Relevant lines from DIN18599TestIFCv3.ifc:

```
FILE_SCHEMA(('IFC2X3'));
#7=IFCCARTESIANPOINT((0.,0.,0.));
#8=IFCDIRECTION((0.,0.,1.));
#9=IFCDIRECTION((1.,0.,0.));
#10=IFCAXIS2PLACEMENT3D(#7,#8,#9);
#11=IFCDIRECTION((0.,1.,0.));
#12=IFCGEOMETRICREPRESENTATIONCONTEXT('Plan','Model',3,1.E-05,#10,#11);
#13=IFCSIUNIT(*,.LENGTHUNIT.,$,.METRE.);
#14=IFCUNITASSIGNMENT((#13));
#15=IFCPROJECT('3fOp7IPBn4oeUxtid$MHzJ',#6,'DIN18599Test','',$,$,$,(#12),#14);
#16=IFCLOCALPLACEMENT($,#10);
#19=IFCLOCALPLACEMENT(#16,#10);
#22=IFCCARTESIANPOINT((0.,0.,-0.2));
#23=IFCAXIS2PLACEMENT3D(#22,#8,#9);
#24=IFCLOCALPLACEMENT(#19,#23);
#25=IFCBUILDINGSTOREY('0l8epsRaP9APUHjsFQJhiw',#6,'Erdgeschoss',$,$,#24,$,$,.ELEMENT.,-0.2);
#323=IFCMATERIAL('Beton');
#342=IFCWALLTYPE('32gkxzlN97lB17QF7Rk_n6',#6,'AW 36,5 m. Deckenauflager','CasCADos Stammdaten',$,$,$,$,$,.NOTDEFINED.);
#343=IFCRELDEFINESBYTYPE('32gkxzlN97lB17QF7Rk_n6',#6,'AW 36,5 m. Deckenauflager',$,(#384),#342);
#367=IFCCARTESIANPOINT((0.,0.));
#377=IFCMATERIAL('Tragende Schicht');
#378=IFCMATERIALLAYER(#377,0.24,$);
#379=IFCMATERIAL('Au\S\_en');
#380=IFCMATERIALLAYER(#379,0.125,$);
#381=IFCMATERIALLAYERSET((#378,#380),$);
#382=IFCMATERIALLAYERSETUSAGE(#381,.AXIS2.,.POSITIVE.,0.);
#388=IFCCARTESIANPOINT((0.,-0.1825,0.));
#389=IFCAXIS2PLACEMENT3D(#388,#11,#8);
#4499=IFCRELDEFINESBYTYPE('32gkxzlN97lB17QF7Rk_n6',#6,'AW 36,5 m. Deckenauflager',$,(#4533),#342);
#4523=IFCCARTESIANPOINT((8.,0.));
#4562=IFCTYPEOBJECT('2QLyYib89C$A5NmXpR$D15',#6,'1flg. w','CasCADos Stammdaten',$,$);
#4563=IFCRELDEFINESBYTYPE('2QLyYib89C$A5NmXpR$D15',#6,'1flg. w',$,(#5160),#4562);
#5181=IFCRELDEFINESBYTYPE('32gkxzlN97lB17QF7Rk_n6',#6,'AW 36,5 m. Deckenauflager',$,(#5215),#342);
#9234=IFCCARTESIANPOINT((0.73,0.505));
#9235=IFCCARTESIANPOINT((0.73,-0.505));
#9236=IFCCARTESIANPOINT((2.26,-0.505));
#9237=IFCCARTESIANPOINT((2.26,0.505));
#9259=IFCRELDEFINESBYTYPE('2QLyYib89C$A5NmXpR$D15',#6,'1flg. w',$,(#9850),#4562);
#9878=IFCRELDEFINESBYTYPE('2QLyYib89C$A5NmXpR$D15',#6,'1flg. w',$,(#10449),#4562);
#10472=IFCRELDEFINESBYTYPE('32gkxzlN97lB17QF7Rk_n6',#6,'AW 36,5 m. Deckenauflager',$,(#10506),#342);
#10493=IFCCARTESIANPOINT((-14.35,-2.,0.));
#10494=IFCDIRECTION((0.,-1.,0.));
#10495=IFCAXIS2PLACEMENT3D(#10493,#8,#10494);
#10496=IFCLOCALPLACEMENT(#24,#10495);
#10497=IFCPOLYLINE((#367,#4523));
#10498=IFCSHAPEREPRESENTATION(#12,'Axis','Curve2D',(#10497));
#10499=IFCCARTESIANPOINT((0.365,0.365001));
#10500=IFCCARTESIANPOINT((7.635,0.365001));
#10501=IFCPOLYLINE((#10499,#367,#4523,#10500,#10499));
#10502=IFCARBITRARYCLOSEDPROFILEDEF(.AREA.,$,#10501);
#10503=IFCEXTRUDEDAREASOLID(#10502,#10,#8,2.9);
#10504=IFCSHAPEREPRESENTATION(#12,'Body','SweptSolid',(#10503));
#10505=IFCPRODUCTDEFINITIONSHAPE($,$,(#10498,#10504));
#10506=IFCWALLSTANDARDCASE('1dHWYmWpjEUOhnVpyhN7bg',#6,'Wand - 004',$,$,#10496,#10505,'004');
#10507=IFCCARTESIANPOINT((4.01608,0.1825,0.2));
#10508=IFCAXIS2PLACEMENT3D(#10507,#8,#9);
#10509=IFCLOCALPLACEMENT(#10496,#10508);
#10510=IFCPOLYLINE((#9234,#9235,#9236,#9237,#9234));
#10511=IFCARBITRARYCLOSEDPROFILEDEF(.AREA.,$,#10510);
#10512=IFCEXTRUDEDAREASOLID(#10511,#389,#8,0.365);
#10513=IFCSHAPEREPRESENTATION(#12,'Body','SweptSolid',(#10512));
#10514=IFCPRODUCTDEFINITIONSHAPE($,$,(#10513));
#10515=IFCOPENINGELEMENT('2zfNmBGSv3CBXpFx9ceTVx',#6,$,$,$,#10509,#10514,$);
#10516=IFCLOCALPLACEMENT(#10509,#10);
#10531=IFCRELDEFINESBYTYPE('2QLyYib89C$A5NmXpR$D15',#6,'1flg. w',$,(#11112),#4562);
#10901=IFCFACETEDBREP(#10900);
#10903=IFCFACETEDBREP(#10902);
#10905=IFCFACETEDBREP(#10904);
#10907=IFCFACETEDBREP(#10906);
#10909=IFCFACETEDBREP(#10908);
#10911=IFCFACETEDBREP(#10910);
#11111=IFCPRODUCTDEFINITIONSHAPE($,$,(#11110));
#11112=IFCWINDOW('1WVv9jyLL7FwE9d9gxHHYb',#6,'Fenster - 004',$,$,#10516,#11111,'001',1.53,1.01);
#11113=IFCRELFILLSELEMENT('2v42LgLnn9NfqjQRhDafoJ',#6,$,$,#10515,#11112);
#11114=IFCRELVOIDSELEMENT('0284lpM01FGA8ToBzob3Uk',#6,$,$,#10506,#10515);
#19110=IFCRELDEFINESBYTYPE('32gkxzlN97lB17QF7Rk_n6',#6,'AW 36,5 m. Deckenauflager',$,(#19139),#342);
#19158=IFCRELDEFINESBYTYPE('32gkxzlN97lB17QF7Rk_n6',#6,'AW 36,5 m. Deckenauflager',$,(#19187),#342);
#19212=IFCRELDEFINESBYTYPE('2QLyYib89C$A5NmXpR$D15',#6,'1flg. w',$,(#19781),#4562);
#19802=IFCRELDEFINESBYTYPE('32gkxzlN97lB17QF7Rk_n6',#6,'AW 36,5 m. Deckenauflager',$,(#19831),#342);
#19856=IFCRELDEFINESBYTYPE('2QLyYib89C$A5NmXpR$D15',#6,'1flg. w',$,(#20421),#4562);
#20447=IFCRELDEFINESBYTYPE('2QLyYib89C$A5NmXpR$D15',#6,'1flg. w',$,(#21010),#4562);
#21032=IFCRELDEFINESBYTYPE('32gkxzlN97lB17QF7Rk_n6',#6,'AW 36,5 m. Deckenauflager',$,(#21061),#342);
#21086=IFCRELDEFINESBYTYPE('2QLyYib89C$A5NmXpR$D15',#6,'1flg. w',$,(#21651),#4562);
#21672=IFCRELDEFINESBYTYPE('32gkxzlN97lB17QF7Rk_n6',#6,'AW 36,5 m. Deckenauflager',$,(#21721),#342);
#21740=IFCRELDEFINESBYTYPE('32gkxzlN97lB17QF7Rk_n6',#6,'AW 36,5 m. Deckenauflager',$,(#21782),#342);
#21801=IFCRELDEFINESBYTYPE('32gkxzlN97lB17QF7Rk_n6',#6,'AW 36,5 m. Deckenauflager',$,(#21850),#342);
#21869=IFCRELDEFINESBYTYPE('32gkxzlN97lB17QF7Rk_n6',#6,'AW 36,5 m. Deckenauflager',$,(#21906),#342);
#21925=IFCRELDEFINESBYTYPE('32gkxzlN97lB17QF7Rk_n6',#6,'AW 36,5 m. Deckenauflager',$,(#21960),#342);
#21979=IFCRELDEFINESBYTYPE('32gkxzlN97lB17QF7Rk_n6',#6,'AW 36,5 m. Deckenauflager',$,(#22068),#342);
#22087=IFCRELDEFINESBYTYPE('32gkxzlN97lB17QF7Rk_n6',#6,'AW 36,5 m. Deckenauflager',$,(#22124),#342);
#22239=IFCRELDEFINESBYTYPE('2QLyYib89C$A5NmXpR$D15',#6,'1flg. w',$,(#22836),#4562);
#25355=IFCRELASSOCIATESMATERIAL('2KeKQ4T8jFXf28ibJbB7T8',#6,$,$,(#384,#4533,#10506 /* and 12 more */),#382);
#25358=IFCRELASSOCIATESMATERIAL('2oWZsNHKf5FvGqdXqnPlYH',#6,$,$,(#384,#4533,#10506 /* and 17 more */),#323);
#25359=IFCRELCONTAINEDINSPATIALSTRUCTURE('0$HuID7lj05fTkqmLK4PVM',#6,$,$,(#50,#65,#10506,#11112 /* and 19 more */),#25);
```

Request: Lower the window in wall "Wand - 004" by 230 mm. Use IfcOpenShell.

```python
import numpy as np
import ifcopenshell
import ifcopenshell.api.geometry
import ifcopenshell.util.placement
import ifcopenshell.util.unit

model = ifcopenshell.open("DIN18599TestIFCv3.ifc")
unit_scale = ifcopenshell.util.unit.calculate_unit_scale(model)

window = model.by_guid("1WVv9jyLL7FwE9d9gxHHYb")
opening = window.FillsVoids[0].RelatingOpeningElement
dz = -0.23 / unit_scale

shift = np.array([0.0, 0.0, dz])
# The window is placed relative to its opening, so it follows when the opening moves.
matrix = ifcopenshell.util.placement.get_local_placement(opening.ObjectPlacement)
matrix[:3, 3] += shift
ifcopenshell.api.geometry.edit_object_placement(
    model, product=opening, matrix=matrix, is_si=False, should_transform_children=True
)

print(f"moved by {dz * unit_scale:+.3f} m")

model.write("DIN18599TestIFCv3_updated.ifc")
```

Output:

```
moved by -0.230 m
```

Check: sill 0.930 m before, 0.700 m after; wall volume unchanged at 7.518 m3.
